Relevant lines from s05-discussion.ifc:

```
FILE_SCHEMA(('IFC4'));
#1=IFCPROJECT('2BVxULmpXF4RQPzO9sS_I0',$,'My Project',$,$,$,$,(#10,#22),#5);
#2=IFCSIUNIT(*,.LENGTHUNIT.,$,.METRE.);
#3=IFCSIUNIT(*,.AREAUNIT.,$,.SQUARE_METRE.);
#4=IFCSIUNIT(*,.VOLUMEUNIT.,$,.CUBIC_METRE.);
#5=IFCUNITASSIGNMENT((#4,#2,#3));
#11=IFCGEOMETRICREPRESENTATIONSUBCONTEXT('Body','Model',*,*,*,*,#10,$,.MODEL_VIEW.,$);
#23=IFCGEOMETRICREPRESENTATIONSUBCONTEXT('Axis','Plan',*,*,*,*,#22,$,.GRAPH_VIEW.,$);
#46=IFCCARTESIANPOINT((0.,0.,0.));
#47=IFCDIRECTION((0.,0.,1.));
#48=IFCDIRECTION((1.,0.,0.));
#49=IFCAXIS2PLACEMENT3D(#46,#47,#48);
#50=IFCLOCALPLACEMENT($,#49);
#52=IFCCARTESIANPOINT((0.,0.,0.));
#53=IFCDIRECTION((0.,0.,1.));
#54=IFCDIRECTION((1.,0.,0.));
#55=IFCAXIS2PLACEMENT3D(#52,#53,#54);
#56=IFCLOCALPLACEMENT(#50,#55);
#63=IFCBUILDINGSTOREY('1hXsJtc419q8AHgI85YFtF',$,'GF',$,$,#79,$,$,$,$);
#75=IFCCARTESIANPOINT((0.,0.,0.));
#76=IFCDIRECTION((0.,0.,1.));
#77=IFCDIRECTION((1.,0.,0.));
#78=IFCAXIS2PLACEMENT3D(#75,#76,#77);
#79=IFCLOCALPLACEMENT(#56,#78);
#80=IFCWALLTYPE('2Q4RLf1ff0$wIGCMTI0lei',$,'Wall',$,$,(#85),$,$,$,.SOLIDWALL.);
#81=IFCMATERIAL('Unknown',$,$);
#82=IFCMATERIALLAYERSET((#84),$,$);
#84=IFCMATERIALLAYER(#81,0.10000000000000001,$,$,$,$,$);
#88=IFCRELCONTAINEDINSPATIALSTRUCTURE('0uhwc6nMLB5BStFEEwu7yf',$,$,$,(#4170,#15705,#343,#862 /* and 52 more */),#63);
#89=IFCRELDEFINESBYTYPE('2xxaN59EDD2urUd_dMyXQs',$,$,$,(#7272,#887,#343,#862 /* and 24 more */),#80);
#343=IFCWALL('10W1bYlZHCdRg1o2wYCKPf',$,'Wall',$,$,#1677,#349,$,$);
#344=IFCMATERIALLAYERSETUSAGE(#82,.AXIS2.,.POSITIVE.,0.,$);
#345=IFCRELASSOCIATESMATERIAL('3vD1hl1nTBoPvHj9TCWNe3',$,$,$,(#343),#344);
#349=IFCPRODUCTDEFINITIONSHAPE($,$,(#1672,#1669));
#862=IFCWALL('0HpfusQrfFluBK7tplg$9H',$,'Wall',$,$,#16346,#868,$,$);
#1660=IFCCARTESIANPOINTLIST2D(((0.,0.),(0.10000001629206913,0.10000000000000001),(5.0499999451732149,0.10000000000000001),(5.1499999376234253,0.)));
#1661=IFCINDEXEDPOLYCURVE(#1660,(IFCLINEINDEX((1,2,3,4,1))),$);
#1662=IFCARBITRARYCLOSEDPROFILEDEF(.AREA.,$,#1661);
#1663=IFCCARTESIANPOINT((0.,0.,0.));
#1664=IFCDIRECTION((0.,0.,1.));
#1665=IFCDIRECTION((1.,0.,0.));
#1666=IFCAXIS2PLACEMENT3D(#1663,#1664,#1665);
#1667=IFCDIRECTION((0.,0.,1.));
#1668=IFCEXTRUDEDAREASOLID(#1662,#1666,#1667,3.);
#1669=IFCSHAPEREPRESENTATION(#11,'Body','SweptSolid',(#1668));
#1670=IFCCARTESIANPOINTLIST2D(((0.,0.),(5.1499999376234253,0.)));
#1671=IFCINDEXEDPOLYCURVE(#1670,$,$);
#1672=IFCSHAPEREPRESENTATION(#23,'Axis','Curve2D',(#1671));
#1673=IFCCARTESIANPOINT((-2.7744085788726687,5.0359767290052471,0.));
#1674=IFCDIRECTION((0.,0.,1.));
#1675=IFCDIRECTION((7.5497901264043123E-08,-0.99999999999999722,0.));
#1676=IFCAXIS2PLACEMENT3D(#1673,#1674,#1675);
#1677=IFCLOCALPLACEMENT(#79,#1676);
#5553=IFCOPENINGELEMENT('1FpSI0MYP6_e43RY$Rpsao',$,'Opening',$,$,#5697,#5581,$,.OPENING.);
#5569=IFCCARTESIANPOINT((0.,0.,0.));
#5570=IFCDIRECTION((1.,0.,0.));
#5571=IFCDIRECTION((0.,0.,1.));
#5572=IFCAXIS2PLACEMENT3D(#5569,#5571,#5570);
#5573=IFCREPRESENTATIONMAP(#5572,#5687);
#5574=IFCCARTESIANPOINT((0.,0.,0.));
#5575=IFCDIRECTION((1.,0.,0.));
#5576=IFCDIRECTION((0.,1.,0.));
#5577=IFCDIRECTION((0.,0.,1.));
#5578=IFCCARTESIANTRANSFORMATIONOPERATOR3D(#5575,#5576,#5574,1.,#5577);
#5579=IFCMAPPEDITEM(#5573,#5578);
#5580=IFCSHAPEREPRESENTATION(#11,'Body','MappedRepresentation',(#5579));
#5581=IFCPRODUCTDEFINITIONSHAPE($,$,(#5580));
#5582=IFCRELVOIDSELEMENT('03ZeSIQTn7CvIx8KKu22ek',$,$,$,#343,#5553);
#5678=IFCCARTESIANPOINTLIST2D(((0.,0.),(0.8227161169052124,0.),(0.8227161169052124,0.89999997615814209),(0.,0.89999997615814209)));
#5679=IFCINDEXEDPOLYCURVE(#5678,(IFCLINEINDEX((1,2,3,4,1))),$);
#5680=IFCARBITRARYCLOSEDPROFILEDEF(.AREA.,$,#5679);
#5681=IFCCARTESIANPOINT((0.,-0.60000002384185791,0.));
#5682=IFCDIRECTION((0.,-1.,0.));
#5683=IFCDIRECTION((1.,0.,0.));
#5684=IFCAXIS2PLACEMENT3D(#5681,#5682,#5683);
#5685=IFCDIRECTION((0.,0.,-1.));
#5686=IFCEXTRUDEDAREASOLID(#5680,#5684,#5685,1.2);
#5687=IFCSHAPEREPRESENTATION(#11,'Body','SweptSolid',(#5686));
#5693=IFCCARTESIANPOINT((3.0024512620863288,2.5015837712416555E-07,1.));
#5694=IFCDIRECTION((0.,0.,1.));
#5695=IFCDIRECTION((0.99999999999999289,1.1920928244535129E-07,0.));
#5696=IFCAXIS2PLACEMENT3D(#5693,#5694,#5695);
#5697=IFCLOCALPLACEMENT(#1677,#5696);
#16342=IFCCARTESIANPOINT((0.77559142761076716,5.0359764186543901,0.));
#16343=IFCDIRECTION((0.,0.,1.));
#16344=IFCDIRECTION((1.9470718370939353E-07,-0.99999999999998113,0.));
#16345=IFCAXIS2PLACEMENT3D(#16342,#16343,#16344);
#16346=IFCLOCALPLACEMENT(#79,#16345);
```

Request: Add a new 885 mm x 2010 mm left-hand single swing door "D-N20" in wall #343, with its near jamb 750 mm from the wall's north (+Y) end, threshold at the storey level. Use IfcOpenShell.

```python
import numpy as np
import ifcopenshell
import ifcopenshell.api.feature
import ifcopenshell.api.geometry
import ifcopenshell.api.root
import ifcopenshell.api.spatial
import ifcopenshell.geom
import ifcopenshell.util.element
import ifcopenshell.util.placement
import ifcopenshell.util.representation
import ifcopenshell.util.shape
import ifcopenshell.util.unit

model = ifcopenshell.open("s05-discussion.ifc")
unit_scale = ifcopenshell.util.unit.calculate_unit_scale(model)
settings = ifcopenshell.geom.settings()


def volume(element):
    """Net volume in cubic metres, openings subtracted."""
    shape = ifcopenshell.geom.create_shape(settings, element)
    return ifcopenshell.util.shape.get_volume(shape.geometry)


wall = model.by_guid("10W1bYlZHCdRg1o2wYCKPf")
storey = ifcopenshell.util.element.get_container(wall, ifc_class="IfcBuildingStorey")
context = ifcopenshell.util.representation.get_context(model, "Model", "Body", "MODEL_VIEW")
before = volume(wall)

width, height, from_end, sill = 0.885, 2.01, 0.75, 0.0  # metres

# The wall runs along its own X axis, and the end named is its -X end.
wall_shape = ifcopenshell.geom.create_shape(settings, wall)
x, y, z = ifcopenshell.util.shape.get_vertices(wall_shape.geometry).T
start = x.min() + from_end
face, thickness = float(y.min()), float(y.max() - y.min())
wall_matrix = ifcopenshell.util.placement.get_local_placement(wall.ObjectPlacement)
level = ifcopenshell.util.placement.get_local_placement(storey.ObjectPlacement)[2, 3]


def in_wall(x, y):
    """Placement at x, y metres in the wall's axes, at sill height."""
    matrix = wall_matrix.copy()
    matrix[:, 3] = wall_matrix @ np.array([x / unit_scale, y / unit_scale, 0.0, 1.0])
    matrix[2, 3] = level + sill / unit_scale
    return matrix


# Opening: a box that overshoots both wall faces by 50 mm.
opening = ifcopenshell.api.root.create_entity(model, ifc_class="IfcOpeningElement", predefined_type="OPENING")
box = ifcopenshell.api.geometry.add_wall_representation(
    model, context=context, length=width, height=height, thickness=thickness + 0.1
)
ifcopenshell.api.geometry.assign_representation(model, product=opening, representation=box)
ifcopenshell.api.geometry.edit_object_placement(model, product=opening, matrix=in_wall(start, face - 0.05), is_si=False)
ifcopenshell.api.feature.add_feature(model, feature=opening, element=wall)

door = ifcopenshell.api.root.create_entity(model, ifc_class="IfcDoor", name="D-N20", predefined_type="DOOR")
door.OverallWidth, door.OverallHeight = width / unit_scale, height / unit_scale
door.OperationType = "SINGLE_SWING_LEFT"
body = ifcopenshell.api.geometry.add_door_representation(
    model,
    context=context,
    overall_width=door.OverallWidth,
    overall_height=door.OverallHeight,
    operation_type="SINGLE_SWING_LEFT",
    lining_properties={"LiningDepth": thickness / unit_scale, "ThresholdDepth": thickness / unit_scale},
)
ifcopenshell.api.geometry.assign_representation(model, product=door, representation=body)
ifcopenshell.api.spatial.assign_container(model, products=[door], relating_structure=storey)
ifcopenshell.api.feature.add_filling(model, opening=opening, element=door)

# The lining spans the wall, so the door starts at the wall face.
ifcopenshell.api.geometry.edit_object_placement(model, product=door, matrix=in_wall(start, face), is_si=False)

after = volume(wall)

print(f"wall volume {before:.3f} -> {after:.3f} m3")

model.write("s05-discussion_rev.ifc")
```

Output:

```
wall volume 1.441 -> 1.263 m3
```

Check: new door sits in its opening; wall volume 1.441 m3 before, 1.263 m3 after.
